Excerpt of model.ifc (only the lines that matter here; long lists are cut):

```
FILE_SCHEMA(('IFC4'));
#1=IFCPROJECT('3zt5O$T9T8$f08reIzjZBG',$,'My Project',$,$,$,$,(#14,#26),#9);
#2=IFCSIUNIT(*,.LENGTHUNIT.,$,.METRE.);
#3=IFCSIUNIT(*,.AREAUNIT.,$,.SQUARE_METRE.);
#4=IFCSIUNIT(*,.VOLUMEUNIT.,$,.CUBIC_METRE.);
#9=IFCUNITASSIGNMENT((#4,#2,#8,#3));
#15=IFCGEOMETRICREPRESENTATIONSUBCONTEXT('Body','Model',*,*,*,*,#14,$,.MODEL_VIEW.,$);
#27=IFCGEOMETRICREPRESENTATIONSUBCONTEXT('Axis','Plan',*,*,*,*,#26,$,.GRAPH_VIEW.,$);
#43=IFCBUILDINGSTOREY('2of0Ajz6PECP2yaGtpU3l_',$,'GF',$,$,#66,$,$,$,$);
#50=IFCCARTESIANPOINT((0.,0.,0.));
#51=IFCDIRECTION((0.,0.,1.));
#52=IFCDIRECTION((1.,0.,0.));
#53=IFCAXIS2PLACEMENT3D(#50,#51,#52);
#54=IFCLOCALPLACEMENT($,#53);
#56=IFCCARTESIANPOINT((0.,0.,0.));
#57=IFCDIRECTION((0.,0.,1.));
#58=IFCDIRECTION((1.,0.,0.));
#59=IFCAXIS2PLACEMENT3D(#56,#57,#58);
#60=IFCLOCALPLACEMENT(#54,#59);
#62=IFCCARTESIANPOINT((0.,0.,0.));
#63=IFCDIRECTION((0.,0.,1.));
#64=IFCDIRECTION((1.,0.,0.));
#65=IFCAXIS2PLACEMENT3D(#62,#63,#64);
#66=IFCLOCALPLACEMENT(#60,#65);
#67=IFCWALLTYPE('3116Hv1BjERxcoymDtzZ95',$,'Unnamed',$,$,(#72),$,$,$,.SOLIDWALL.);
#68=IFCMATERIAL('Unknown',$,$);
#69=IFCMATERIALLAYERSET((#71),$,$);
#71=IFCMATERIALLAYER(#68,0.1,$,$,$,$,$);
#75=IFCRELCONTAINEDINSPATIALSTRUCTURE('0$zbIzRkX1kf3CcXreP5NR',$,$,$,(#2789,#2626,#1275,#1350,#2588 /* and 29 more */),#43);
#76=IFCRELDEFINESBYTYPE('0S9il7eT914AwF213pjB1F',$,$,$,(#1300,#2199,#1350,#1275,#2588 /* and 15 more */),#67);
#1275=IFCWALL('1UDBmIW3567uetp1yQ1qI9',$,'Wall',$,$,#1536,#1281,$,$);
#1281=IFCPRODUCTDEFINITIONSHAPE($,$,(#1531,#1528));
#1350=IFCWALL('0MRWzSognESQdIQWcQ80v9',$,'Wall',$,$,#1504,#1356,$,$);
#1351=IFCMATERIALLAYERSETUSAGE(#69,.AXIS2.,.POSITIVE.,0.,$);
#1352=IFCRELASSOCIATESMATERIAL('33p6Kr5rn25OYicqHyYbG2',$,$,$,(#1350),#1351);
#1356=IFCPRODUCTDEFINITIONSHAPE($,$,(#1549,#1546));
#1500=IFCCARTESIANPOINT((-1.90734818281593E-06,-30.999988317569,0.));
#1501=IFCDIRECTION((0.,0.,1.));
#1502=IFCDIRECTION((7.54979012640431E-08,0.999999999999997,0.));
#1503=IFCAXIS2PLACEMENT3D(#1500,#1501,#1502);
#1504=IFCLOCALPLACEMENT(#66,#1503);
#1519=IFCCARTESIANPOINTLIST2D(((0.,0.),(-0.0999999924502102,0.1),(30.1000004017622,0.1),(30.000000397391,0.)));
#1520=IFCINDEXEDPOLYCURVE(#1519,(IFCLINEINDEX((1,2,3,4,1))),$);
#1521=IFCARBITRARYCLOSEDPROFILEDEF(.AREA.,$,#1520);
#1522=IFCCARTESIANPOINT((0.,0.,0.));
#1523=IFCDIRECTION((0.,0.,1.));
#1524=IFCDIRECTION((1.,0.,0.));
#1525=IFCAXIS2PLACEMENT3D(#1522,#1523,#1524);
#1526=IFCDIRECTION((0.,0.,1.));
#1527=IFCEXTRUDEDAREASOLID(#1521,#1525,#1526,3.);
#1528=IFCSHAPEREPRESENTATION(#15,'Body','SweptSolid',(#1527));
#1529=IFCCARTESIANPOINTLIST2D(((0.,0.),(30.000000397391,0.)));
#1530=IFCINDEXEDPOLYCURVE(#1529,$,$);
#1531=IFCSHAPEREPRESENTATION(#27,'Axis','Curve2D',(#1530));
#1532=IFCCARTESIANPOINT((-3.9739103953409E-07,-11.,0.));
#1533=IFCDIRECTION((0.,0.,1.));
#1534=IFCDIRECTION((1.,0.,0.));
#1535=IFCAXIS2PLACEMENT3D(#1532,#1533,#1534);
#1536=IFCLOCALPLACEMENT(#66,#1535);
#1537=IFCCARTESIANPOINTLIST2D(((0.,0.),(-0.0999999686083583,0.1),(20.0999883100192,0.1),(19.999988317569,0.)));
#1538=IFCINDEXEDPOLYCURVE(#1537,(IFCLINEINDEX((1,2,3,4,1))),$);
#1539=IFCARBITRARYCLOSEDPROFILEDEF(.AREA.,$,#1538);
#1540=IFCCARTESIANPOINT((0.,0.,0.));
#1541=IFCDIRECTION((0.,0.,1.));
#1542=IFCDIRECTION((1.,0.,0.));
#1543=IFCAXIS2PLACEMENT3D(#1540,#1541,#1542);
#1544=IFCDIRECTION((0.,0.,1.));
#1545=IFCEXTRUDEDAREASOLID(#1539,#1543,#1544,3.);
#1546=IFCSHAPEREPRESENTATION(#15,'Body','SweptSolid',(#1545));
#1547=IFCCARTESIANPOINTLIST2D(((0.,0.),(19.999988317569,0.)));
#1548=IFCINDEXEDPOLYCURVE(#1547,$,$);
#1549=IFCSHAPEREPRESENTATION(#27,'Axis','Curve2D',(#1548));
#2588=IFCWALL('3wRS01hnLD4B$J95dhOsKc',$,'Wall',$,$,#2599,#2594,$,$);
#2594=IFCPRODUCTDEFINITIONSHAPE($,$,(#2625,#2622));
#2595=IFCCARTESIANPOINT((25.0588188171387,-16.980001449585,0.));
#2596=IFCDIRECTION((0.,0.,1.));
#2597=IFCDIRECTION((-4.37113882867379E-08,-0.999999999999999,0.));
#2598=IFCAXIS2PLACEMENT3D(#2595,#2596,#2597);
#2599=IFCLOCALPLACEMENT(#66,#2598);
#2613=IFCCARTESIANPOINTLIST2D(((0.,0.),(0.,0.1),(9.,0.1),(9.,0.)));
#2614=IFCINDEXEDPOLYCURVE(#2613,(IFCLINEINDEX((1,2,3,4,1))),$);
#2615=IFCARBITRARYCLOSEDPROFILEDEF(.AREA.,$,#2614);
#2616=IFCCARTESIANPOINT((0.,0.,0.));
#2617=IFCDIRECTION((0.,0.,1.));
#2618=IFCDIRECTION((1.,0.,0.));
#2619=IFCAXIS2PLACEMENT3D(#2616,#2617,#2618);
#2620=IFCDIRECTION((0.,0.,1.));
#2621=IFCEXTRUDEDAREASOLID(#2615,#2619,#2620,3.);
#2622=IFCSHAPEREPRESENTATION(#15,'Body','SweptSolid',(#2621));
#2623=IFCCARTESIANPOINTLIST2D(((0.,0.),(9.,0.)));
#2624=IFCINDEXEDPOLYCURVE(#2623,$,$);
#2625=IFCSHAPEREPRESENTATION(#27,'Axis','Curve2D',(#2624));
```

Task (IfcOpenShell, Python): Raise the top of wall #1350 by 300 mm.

```python
import ifcopenshell
import ifcopenshell.geom
import ifcopenshell.util.representation
import ifcopenshell.util.shape
import ifcopenshell.util.unit

model = ifcopenshell.open("model.ifc")
unit_scale = ifcopenshell.util.unit.calculate_unit_scale(model)
settings = ifcopenshell.geom.settings()


def volume(element):
    """Net volume in cubic metres, openings subtracted."""
    shape = ifcopenshell.geom.create_shape(settings, element)
    return ifcopenshell.util.shape.get_volume(shape.geometry)


wall = model.by_guid("0MRWzSognESQdIQWcQ80v9")
before = volume(wall)

body = ifcopenshell.util.representation.get_representation(wall, "Model", "Body")
solid = body.Items[0]
old_height = solid.Depth
solid.Depth += 0.3 / unit_scale
after = volume(wall)

print(f"height {old_height:g} -> {solid.Depth:g}, volume {before:.3f} -> {after:.3f} m3")

model.write("model-out.ifc")
```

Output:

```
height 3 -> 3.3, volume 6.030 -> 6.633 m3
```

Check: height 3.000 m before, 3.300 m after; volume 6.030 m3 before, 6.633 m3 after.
